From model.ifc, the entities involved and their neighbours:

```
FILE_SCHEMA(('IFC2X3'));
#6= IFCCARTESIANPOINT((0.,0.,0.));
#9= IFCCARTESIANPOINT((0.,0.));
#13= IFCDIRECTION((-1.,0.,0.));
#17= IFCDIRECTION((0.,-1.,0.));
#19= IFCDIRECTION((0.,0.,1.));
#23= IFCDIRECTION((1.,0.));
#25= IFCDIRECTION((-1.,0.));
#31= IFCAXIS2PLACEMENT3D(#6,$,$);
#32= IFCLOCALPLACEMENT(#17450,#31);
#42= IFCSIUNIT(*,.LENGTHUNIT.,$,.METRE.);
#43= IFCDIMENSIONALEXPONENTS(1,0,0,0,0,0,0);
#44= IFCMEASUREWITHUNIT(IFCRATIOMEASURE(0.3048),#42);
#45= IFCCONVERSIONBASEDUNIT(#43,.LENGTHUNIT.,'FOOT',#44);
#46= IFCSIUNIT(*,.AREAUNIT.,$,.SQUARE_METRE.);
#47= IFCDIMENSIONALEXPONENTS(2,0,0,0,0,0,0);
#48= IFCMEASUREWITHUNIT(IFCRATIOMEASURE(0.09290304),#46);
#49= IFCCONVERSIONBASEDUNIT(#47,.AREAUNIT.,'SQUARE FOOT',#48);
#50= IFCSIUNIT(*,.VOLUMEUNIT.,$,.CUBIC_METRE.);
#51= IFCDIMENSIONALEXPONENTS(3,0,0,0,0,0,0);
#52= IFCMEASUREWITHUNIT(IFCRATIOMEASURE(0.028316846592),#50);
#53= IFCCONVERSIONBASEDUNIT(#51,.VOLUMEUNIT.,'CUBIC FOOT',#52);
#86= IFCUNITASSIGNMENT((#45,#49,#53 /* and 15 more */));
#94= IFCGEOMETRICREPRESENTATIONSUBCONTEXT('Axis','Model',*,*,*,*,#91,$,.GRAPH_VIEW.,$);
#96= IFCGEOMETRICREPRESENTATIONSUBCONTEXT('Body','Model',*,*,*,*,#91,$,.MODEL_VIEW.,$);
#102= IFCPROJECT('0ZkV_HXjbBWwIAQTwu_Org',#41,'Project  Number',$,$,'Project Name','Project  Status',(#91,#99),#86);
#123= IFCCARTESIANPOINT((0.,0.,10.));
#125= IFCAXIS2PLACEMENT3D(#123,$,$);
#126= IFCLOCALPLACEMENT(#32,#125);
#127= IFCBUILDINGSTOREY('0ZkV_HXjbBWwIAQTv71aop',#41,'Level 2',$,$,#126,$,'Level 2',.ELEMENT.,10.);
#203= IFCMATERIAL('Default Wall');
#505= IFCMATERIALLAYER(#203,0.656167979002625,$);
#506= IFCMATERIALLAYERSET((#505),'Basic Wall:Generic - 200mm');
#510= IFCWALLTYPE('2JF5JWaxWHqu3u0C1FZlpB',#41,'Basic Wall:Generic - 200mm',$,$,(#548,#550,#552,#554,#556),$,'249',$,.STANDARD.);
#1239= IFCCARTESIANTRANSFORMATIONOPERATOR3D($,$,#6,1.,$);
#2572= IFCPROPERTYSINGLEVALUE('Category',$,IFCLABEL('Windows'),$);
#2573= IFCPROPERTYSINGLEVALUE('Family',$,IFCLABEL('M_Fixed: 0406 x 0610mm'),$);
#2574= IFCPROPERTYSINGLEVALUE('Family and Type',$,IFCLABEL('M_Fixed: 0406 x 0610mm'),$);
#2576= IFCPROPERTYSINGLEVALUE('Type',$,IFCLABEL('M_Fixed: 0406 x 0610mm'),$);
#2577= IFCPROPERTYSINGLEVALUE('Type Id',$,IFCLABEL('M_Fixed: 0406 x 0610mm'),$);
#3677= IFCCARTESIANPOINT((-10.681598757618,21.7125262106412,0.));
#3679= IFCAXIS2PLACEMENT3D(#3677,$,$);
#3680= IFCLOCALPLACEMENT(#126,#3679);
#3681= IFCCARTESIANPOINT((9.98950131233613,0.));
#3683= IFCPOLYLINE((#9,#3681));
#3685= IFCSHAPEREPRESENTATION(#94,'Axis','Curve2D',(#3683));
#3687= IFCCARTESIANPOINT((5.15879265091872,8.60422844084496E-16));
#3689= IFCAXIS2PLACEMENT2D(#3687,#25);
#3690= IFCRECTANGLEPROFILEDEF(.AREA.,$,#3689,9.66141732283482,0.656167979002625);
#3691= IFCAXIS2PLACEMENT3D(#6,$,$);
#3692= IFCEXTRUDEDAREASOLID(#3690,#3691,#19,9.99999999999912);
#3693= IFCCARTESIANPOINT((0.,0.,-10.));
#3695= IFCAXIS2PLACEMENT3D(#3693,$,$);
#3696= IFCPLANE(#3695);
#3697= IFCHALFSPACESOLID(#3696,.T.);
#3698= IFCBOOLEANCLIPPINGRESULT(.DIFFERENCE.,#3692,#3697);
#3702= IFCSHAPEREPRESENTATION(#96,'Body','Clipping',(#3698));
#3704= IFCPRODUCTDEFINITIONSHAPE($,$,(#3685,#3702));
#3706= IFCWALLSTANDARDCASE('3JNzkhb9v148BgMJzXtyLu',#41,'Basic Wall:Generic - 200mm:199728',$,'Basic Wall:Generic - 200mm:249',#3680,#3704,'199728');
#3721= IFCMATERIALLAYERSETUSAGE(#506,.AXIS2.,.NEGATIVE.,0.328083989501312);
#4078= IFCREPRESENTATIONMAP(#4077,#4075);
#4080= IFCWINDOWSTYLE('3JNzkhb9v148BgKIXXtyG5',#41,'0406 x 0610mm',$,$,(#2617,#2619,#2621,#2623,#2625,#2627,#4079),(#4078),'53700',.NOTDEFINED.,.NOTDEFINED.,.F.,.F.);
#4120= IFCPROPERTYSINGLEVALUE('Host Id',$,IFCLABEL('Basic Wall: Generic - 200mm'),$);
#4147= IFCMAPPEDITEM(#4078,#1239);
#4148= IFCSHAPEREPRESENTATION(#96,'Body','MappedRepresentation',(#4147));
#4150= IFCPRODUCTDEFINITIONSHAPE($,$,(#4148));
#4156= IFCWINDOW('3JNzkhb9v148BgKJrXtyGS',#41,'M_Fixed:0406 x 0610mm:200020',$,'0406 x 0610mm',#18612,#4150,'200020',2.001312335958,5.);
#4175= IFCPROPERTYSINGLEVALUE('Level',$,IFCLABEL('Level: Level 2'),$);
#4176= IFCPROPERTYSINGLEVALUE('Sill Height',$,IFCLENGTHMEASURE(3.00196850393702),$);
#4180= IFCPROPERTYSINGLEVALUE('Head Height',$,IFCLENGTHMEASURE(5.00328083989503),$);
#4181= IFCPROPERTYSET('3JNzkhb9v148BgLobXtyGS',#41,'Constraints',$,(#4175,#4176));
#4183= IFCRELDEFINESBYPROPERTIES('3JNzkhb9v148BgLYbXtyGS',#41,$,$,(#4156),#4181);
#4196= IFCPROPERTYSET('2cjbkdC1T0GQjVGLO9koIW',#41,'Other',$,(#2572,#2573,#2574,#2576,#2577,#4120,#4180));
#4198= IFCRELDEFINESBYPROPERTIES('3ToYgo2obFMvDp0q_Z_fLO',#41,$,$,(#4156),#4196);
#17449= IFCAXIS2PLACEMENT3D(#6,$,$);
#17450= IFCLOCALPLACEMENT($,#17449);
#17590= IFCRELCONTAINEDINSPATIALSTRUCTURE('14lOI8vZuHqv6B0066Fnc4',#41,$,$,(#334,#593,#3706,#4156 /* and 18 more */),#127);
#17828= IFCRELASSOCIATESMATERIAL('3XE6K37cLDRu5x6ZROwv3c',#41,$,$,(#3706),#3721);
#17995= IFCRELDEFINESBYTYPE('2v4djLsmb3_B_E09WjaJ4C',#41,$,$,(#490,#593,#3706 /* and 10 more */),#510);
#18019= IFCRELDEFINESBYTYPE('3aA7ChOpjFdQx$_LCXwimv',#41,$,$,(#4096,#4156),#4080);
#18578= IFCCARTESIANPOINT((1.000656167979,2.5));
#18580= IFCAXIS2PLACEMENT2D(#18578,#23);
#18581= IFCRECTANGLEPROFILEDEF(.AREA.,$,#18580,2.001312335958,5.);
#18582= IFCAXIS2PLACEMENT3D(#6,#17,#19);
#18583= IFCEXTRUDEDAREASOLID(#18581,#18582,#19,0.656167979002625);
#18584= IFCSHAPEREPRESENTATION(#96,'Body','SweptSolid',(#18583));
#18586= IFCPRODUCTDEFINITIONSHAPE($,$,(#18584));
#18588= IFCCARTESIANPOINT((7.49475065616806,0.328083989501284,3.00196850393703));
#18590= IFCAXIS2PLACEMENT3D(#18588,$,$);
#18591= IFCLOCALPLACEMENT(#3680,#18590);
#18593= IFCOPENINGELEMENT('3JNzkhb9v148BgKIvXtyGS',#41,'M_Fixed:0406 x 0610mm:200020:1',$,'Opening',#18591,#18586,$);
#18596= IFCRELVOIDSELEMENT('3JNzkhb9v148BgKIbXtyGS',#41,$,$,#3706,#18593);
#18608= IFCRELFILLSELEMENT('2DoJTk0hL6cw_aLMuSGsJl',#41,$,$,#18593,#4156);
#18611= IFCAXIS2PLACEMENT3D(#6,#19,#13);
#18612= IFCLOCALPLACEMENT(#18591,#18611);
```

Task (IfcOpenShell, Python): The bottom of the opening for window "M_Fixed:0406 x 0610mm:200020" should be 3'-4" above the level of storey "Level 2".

```python
import numpy as np
import ifcopenshell
import ifcopenshell.api.geometry
import ifcopenshell.api.pset
import ifcopenshell.geom
import ifcopenshell.util.element
import ifcopenshell.util.placement
import ifcopenshell.util.shape
import ifcopenshell.util.unit

model = ifcopenshell.open("model.ifc")
unit_scale = ifcopenshell.util.unit.calculate_unit_scale(model)

window = model.by_guid("3JNzkhb9v148BgKJrXtyGS")
opening = window.FillsVoids[0].RelatingOpeningElement
storey = ifcopenshell.util.element.get_container(window, ifc_class="IfcBuildingStorey")
level = ifcopenshell.util.placement.get_local_placement(storey.ObjectPlacement)[2, 3]

# The opening's origin need not be at the sill, so measure its lowest point.
shape = ifcopenshell.geom.create_shape(ifcopenshell.geom.settings(), opening)
bottom = ifcopenshell.util.shape.get_shape_bottom_elevation(shape, shape.geometry) / unit_scale
dz = level + 40 * 0.0254 / unit_scale - bottom

shift = np.array([0.0, 0.0, dz])
# The window is placed relative to its opening, so it follows when the opening moves.
matrix = ifcopenshell.util.placement.get_local_placement(opening.ObjectPlacement)
matrix[:3, 3] += shift
ifcopenshell.api.geometry.edit_object_placement(
    model, product=opening, matrix=matrix, is_si=False, should_transform_children=True
)

# Keep the stored heights in step.
pset = model.by_id(ifcopenshell.util.element.get_pset(window, "Constraints", should_inherit=False)["id"])
ifcopenshell.api.pset.edit_pset(model, pset=pset, properties={
    "Sill Height": model.create_entity("IfcLengthMeasure", ifcopenshell.util.element.get_pset(window, "Constraints", "Sill Height") + dz),
})
pset = model.by_id(ifcopenshell.util.element.get_pset(window, "Other", should_inherit=False)["id"])
ifcopenshell.api.pset.edit_pset(model, pset=pset, properties={
    "Head Height": model.create_entity("IfcLengthMeasure", ifcopenshell.util.element.get_pset(window, "Other", "Head Height") + dz),
})

print(f"moved by {dz * unit_scale:+.3f} m")

model.write("model_rev.ifc")
```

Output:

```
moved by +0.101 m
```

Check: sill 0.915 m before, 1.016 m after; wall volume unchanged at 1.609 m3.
